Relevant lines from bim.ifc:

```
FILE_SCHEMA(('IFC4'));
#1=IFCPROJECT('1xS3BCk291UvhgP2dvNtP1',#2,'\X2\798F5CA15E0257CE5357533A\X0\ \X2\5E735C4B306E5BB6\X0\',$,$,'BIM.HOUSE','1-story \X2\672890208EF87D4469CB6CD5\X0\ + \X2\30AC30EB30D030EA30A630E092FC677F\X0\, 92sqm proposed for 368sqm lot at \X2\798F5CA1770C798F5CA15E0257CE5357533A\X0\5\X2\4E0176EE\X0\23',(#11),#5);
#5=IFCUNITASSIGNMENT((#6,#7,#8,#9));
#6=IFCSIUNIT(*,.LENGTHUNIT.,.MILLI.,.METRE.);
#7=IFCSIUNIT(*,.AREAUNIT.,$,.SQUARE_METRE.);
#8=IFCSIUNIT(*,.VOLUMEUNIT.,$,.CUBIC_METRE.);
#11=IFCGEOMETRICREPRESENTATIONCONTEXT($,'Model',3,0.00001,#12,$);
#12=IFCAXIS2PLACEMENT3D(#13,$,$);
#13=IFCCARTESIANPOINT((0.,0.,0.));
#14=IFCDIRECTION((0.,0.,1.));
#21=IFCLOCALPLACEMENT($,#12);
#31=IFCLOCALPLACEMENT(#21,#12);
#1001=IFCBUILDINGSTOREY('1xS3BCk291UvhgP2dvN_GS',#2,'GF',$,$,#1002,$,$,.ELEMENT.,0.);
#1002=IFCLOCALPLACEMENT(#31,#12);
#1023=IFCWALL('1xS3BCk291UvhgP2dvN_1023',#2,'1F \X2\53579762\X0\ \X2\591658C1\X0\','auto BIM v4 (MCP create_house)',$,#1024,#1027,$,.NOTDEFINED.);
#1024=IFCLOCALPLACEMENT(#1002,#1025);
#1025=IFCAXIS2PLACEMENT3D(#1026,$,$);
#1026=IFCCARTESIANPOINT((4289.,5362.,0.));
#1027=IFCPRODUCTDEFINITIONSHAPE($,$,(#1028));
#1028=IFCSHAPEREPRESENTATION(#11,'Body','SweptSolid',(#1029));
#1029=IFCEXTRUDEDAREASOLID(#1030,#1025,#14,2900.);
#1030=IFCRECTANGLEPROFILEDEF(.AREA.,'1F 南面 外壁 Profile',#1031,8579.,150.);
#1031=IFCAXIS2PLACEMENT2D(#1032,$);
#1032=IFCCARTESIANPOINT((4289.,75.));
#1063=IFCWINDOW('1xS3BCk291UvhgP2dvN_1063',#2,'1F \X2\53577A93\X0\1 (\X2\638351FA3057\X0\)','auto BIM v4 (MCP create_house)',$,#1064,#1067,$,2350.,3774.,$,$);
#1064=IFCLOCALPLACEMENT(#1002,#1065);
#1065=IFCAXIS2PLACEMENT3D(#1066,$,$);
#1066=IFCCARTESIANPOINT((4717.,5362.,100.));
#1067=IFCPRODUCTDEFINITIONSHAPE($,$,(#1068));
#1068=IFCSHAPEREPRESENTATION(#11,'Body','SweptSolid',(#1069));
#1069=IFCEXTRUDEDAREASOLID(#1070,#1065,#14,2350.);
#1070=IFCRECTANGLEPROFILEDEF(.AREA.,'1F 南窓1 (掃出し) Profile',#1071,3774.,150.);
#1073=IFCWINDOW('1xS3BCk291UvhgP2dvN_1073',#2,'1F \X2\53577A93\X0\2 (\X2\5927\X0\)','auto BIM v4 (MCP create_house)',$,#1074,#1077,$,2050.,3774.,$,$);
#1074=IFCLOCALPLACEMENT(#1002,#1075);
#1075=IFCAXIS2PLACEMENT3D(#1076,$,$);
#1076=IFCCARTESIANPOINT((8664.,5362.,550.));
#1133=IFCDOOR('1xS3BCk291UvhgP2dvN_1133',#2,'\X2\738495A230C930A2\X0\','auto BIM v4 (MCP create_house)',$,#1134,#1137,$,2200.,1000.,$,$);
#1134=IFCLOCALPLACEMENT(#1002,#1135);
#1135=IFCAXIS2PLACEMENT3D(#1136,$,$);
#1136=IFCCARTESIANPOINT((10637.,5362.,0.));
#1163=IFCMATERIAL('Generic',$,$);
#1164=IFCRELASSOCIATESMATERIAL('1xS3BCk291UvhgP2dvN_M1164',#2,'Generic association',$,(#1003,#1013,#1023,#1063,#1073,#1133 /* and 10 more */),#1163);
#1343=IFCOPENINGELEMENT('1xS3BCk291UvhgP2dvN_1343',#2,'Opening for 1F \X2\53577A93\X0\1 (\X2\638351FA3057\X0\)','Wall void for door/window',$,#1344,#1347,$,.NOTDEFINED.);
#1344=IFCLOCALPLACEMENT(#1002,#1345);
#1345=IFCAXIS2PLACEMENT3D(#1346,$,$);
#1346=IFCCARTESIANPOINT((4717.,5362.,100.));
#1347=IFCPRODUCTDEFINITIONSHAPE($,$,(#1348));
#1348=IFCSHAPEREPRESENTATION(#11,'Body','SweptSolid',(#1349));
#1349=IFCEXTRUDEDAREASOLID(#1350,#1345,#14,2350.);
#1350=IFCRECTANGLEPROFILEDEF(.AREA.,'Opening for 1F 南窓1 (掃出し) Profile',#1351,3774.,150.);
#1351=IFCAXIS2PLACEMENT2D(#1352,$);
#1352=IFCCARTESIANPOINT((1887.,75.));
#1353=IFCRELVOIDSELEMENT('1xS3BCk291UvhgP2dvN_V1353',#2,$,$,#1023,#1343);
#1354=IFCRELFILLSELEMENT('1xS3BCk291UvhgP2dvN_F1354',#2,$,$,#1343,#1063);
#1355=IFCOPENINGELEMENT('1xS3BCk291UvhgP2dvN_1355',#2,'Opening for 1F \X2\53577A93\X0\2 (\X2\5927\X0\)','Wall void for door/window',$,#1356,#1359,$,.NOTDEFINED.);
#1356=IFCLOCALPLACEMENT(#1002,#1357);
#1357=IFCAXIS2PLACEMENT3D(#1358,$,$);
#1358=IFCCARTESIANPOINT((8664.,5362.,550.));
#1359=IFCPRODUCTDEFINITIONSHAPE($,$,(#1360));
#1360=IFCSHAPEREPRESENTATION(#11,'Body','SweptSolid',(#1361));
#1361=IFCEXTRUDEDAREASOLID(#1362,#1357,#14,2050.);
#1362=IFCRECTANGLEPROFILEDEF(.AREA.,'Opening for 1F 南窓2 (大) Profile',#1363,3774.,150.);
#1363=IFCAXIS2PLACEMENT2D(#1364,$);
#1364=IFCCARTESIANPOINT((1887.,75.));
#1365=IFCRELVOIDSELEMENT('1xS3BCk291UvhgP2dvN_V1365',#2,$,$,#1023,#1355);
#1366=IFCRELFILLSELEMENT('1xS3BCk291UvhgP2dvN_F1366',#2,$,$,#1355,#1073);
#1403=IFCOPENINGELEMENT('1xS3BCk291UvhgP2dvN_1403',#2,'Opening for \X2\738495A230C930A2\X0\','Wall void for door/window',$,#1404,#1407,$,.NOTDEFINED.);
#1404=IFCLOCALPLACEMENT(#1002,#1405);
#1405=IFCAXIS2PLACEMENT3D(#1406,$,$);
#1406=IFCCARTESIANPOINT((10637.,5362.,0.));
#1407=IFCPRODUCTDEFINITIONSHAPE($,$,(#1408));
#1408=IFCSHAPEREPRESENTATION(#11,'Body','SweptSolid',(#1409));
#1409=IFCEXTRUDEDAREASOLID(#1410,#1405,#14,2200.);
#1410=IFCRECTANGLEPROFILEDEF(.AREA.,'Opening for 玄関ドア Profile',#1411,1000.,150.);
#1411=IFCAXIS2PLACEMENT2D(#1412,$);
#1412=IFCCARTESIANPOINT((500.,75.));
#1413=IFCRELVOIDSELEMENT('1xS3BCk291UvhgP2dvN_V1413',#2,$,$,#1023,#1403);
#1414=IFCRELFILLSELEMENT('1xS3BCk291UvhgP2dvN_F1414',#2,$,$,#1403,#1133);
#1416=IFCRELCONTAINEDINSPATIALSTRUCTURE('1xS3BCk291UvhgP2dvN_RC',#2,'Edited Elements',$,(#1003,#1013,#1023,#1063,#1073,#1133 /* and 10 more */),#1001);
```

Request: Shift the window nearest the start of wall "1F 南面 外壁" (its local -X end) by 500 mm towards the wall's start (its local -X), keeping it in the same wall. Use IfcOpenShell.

```python
import ifcopenshell
import ifcopenshell.api.geometry
import ifcopenshell.util.placement
import ifcopenshell.util.unit

model = ifcopenshell.open("bim.ifc")
unit_scale = ifcopenshell.util.unit.calculate_unit_scale(model)

window = model.by_id(1063)
opening = window.FillsVoids[0].RelatingOpeningElement
wall = opening.VoidsElements[0].RelatingBuildingElement

wall_matrix = ifcopenshell.util.placement.get_local_placement(wall.ObjectPlacement)
shift = wall_matrix[:3, 0] * -0.5 / unit_scale
before = ifcopenshell.util.placement.get_local_placement(window.ObjectPlacement)[:3, 3].copy()

# The window is not placed relative to its opening, so move both.
for product in (opening, window):
    matrix = ifcopenshell.util.placement.get_local_placement(product.ObjectPlacement)
    matrix[:3, 3] += shift
    ifcopenshell.api.geometry.edit_object_placement(model, product=product, matrix=matrix, is_si=False)

after = ifcopenshell.util.placement.get_local_placement(window.ObjectPlacement)[:3, 3]
print("window moved by", (after - before).round(3) + 0.0)

model.write("bim_updated.ifc")
```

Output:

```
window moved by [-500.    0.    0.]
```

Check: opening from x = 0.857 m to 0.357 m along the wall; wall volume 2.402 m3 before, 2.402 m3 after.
